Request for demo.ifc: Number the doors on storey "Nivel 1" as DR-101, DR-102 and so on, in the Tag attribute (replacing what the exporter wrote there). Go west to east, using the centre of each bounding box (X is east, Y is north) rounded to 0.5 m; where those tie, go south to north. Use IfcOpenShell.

First a look at what the model holds.

```python
import ifcopenshell
import ifcopenshell.util.element
import ifcopenshell.util.placement

model = ifcopenshell.open("demo.ifc")
print(model.schema)
storey = next(s for s in model.by_type("IfcBuildingStorey") if s.Name == "Nivel 1")
doors = [e for e in ifcopenshell.util.element.get_decomposition(storey) if e.is_a("IfcDoor")]
for e in sorted(doors, key=lambda e: e.id()):
    origin = ifcopenshell.util.placement.get_local_placement(e.ObjectPlacement)[:3, 3]
    print(e.id(), e.Tag, e.Name, origin.round(2) + 0.0, sep=" | ")
```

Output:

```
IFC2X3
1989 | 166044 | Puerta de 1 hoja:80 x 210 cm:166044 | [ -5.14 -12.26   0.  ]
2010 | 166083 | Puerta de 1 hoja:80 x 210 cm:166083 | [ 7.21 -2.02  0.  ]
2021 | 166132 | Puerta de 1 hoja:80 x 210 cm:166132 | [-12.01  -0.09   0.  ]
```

```python
import ifcopenshell
import ifcopenshell.geom
import ifcopenshell.util.element
import ifcopenshell.util.shape

model = ifcopenshell.open("demo.ifc")
settings = ifcopenshell.geom.settings()
settings.set("use-world-coords", True)


def centre(element):
    shape = ifcopenshell.geom.create_shape(settings, element)
    return ifcopenshell.util.shape.get_bbox_centroid(shape.geometry)


storey = next(s for s in model.by_type("IfcBuildingStorey") if s.Name == "Nivel 1")
doors = [e for e in ifcopenshell.util.element.get_decomposition(storey) if e.is_a("IfcDoor")]

# Insertion points can sit at a corner or the storey origin, so sort by the geometry (in metres).
centres = {e: centre(e) for e in doors}
doors.sort(key=lambda e: (round(centres[e][0] / 0.5), centres[e][1]))

for i, e in enumerate(doors, start=1):
    number = f"DR-1{i:02d}"
    e.Tag = number
    print(e.id(), number)

model.write("demo_updated.ifc")
```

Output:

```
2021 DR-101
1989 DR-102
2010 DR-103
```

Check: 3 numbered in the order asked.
